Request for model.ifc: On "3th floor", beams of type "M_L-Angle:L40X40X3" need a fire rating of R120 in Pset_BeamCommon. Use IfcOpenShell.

First a look at what the model holds.

```python
import ifcopenshell
import ifcopenshell.util.element

model = ifcopenshell.open("model.ifc")
print(model.schema)
storey = next(s for s in model.by_type("IfcBuildingStorey") if s.Name == "3th floor")
beams = [e for e in ifcopenshell.util.element.get_decomposition(storey) if e.is_a("IfcBeam")]
seen = {}
for e in beams:
    element_type = ifcopenshell.util.element.get_type(e)
    key = (element_type.Name if element_type != e and element_type else None, ifcopenshell.util.element.get_pset(e, "Pset_BeamCommon", "FireRating"))
    seen[key] = seen.get(key, 0) + 1
for (name, value), count in sorted(seen.items(), key=str):
    print(count, "x", name, "|", value)
```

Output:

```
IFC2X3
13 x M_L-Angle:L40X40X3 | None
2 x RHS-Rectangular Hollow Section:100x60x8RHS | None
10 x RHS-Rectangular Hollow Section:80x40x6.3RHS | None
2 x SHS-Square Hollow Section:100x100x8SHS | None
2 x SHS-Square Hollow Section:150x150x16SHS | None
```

```python
import ifcopenshell
import ifcopenshell.api.pset
import ifcopenshell.util.element

model = ifcopenshell.open("model.ifc")

storey = next(s for s in model.by_type("IfcBuildingStorey") if s.Name == "3th floor")
beams = [e for e in ifcopenshell.util.element.get_decomposition(storey) if e.is_a("IfcBeam")]

count = 0
for e in beams:
    element_type = ifcopenshell.util.element.get_type(e)
    if element_type in (None, e) or element_type.Name != "M_L-Angle:L40X40X3":
        continue
    # add_pset returns the element's existing set when there is one.
    pset = ifcopenshell.api.pset.add_pset(model, product=e, name="Pset_BeamCommon")
    ifcopenshell.api.pset.edit_pset(model, pset=pset, properties={"FireRating": "R120"})
    count += 1

print(count, "beams updated")

model.write("model_edited.ifc")
```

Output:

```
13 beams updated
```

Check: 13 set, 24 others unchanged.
